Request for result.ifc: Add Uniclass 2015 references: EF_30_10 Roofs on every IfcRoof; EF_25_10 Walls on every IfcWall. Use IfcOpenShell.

First a look at what the model holds.

```python
import ifcopenshell

model = ifcopenshell.open("result.ifc")
print(model.schema)
print("classifications:", [c.Name for c in model.by_type("IfcClassification")])
for ifc_class in ("IfcDoor", "IfcRoof", "IfcStair", "IfcWall", "IfcWindow"):
    print(ifc_class, len(model.by_type(ifc_class)))
```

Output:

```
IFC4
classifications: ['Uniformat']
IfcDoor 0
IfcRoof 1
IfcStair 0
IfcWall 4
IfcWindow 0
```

```python
import ifcopenshell
import ifcopenshell.api.classification

model = ifcopenshell.open("result.ifc")

system = ifcopenshell.api.classification.add_classification(model, classification="Uniclass 2015")

codes = {
    "IfcRoof": ("EF_30_10", "Roofs"),
    "IfcWall": ("EF_25_10", "Walls"),
}
for ifc_class, (code, name) in codes.items():
    products = model.by_type(ifc_class)
    ifcopenshell.api.classification.add_reference(
        model, products=products, classification=system, identification=code, name=name
    )
    print(code, len(products))

model.write("result_updated.ifc")
```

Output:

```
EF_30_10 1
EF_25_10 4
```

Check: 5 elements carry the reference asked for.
